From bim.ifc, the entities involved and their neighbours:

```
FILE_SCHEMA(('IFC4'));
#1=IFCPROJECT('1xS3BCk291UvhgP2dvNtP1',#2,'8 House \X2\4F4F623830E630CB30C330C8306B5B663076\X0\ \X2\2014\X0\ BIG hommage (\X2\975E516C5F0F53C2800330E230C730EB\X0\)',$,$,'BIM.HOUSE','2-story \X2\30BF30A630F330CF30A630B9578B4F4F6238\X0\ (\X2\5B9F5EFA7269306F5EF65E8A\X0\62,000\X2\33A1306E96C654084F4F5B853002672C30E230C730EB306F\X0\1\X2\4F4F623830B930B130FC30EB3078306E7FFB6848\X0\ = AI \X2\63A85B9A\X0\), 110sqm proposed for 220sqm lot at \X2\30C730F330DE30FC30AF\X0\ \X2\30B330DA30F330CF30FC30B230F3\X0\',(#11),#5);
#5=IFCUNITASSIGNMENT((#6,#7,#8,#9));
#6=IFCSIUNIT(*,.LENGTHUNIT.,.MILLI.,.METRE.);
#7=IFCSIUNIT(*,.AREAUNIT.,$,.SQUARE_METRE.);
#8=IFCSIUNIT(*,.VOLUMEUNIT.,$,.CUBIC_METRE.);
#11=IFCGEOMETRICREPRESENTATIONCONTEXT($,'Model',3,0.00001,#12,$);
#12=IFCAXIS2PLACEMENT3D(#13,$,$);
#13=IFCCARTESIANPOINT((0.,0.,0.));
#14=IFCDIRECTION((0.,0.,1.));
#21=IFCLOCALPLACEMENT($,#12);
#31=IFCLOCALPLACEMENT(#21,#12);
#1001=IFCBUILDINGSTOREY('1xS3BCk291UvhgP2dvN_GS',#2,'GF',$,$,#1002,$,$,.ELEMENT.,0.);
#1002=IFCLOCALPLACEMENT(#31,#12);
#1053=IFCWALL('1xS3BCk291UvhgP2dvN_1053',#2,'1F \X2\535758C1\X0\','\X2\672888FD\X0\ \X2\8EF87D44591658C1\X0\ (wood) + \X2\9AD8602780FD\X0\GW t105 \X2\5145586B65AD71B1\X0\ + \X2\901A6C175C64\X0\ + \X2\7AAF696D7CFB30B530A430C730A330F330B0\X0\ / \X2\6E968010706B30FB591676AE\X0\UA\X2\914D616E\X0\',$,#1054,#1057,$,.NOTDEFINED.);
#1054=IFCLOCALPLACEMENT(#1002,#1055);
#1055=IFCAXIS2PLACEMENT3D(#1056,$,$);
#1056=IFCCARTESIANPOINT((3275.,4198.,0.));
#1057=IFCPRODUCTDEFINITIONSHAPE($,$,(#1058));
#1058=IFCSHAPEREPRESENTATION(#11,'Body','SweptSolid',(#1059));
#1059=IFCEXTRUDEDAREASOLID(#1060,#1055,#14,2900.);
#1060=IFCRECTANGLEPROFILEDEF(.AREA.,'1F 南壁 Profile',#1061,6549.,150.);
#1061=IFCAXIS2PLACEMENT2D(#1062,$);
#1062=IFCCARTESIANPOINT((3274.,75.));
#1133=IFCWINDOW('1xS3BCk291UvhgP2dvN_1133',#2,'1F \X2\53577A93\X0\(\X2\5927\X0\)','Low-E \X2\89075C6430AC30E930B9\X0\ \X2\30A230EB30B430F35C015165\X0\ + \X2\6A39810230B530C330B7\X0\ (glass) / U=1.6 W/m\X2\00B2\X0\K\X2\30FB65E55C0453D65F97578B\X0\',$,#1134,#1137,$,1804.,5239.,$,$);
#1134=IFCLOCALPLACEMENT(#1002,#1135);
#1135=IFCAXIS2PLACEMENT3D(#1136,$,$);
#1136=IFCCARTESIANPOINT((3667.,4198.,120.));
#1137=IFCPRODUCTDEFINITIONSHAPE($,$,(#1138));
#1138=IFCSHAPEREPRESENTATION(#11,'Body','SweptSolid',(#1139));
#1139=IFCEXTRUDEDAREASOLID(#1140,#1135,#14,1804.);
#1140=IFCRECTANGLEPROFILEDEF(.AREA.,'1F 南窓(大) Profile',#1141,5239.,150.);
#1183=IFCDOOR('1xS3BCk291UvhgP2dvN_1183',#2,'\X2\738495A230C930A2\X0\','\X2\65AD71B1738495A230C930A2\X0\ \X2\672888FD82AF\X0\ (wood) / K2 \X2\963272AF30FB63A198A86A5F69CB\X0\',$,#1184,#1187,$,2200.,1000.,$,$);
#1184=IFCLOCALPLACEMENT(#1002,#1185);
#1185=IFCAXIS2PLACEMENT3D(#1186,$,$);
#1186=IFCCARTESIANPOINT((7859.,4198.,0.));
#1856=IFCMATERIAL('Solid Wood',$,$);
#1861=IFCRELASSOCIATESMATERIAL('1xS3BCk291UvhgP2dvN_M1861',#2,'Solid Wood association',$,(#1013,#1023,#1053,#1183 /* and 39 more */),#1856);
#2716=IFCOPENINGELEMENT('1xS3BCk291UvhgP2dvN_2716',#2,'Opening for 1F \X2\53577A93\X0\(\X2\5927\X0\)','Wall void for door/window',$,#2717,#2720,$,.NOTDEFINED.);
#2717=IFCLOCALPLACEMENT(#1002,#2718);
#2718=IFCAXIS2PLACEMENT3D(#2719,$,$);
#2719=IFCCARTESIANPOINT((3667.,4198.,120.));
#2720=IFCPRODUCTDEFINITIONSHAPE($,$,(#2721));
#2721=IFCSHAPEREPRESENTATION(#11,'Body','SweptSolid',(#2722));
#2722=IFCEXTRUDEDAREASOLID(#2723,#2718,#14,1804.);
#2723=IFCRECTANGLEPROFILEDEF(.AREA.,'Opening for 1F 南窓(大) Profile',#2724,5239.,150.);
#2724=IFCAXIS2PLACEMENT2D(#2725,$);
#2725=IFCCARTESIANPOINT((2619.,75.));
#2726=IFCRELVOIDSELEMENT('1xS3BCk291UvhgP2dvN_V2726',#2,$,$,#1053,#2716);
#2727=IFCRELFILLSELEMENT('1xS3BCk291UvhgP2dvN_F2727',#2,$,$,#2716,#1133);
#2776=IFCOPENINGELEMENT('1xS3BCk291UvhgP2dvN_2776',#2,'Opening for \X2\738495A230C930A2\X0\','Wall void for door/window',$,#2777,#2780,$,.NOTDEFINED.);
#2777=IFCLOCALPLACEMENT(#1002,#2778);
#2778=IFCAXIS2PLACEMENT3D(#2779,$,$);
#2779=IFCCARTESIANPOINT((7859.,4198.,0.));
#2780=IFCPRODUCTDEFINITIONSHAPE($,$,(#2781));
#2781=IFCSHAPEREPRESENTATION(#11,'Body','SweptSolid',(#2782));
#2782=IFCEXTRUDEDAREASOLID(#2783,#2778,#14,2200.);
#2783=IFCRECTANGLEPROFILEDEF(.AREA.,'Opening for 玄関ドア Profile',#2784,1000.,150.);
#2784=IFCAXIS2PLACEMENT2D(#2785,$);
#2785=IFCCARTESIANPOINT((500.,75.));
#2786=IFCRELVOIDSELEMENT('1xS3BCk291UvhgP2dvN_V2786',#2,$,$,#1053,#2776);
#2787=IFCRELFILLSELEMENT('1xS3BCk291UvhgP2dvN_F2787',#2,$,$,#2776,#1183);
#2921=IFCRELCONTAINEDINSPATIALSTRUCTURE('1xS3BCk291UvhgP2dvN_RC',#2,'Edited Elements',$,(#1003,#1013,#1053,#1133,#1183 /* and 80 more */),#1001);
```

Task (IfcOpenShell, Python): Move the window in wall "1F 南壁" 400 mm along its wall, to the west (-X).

```python
import ifcopenshell
import ifcopenshell.api.geometry
import ifcopenshell.util.placement
import ifcopenshell.util.unit

model = ifcopenshell.open("bim.ifc")
unit_scale = ifcopenshell.util.unit.calculate_unit_scale(model)

window = model.by_id(1133)
opening = window.FillsVoids[0].RelatingOpeningElement
wall = opening.VoidsElements[0].RelatingBuildingElement

wall_matrix = ifcopenshell.util.placement.get_local_placement(wall.ObjectPlacement)
shift = wall_matrix[:3, 0] * -0.4 / unit_scale
before = ifcopenshell.util.placement.get_local_placement(window.ObjectPlacement)[:3, 3].copy()

# The window is not placed relative to its opening, so move both.
for product in (opening, window):
    matrix = ifcopenshell.util.placement.get_local_placement(product.ObjectPlacement)
    matrix[:3, 3] += shift
    ifcopenshell.api.geometry.edit_object_placement(model, product=product, matrix=matrix, is_si=False)

after = ifcopenshell.util.placement.get_local_placement(window.ObjectPlacement)[:3, 3]
print("window moved by", (after - before).round(3) + 0.0)

model.write("bim_updated.ifc")
```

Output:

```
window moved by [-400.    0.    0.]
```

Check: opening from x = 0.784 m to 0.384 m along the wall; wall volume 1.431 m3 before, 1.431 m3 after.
